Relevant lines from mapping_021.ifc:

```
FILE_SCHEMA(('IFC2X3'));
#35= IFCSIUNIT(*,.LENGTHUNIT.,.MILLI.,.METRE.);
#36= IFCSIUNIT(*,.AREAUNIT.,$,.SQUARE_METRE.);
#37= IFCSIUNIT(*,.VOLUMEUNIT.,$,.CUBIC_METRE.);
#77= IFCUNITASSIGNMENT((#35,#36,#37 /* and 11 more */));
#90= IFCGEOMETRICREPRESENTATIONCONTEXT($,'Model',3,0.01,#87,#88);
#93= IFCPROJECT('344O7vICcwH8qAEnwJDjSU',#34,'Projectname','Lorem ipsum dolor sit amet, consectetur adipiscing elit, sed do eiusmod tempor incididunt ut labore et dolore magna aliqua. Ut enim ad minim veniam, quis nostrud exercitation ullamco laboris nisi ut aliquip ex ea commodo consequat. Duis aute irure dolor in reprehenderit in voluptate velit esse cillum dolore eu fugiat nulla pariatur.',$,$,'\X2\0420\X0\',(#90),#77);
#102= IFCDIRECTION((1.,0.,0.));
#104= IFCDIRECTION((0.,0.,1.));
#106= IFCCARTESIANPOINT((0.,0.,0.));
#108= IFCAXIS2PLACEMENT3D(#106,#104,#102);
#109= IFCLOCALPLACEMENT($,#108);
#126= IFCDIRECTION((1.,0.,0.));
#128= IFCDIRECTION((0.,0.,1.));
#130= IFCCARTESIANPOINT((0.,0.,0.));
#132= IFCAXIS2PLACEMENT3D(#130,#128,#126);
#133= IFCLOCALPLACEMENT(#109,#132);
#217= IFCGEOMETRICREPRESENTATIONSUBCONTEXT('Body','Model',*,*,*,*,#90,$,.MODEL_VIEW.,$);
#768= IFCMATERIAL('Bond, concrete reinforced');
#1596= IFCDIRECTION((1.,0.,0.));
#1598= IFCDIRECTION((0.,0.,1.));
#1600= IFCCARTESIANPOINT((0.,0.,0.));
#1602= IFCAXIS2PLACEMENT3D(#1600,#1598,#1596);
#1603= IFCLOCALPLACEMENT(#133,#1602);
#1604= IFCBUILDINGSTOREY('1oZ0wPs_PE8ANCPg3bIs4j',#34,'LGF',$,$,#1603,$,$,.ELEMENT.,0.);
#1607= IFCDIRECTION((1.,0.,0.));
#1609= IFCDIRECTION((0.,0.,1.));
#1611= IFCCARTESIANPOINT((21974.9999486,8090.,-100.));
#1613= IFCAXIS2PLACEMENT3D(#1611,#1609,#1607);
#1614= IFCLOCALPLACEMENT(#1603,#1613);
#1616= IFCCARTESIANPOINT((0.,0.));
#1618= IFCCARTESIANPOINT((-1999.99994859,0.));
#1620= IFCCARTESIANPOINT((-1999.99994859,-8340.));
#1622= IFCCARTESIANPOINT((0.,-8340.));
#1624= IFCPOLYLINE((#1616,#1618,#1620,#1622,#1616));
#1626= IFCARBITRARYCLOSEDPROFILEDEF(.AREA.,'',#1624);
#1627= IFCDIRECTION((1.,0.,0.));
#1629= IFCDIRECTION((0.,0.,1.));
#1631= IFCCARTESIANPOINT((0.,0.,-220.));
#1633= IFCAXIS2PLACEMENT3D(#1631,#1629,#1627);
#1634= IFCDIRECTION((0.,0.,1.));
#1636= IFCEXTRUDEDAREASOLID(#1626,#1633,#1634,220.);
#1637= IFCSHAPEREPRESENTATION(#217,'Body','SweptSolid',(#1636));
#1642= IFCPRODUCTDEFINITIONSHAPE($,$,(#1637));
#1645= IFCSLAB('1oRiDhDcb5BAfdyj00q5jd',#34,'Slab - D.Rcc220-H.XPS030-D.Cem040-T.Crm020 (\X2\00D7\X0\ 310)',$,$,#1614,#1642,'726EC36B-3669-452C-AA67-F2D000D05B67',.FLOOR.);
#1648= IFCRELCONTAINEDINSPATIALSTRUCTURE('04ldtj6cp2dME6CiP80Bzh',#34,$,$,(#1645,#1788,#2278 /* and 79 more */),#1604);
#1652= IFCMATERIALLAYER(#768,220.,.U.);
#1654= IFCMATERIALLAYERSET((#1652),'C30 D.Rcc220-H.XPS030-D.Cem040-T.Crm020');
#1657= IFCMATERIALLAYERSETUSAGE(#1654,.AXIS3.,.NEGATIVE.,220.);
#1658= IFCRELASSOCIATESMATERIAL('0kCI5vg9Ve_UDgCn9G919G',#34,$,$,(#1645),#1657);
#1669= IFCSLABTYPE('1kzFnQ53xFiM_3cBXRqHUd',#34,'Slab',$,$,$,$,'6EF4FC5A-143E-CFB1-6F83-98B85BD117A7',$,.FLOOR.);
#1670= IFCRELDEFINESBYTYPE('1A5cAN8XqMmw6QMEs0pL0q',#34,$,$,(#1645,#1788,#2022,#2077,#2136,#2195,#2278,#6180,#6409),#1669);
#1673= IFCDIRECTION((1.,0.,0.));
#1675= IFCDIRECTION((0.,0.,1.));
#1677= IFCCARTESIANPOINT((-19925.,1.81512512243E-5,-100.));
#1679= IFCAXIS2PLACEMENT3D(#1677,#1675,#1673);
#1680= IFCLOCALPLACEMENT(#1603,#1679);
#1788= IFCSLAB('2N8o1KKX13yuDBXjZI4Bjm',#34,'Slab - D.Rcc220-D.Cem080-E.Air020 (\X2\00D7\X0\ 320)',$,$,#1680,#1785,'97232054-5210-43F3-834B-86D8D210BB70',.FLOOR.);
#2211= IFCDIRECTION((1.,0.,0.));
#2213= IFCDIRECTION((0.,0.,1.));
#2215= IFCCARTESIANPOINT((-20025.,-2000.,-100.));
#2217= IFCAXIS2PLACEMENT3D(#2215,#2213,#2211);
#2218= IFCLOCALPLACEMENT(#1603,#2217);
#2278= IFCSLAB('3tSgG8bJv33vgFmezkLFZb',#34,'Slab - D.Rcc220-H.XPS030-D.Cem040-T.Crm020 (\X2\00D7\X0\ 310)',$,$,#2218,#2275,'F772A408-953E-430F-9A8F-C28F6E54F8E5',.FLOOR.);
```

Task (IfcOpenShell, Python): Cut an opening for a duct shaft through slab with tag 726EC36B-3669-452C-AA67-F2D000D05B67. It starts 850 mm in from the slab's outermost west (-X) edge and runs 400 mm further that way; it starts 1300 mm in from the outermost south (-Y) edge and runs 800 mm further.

```python
import numpy as np
import ifcopenshell
import ifcopenshell.api.feature
import ifcopenshell.api.geometry
import ifcopenshell.api.root
import ifcopenshell.geom
import ifcopenshell.util.placement
import ifcopenshell.util.representation
import ifcopenshell.util.shape
import ifcopenshell.util.unit

model = ifcopenshell.open("mapping_021.ifc")
unit_scale = ifcopenshell.util.unit.calculate_unit_scale(model)
settings = ifcopenshell.geom.settings()


def volume(element):
    """Net volume in cubic metres, openings subtracted."""
    shape = ifcopenshell.geom.create_shape(settings, element)
    return ifcopenshell.util.shape.get_volume(shape.geometry)


slab = model.by_id(1645)
before = volume(slab)

# Extent in the slab's own axes, in metres. The edges named are its -X and -Y sides.
slab_shape = ifcopenshell.geom.create_shape(settings, slab)
vertices = ifcopenshell.util.shape.get_vertices(slab_shape.geometry)
x_min, y_min, bottom = vertices.min(axis=0)
top = vertices[:, 2].max()

opening = ifcopenshell.api.root.create_entity(model, ifc_class="IfcOpeningElement", name="Duct shaft opening")
context = ifcopenshell.util.representation.get_context(model, "Model", "Body", "MODEL_VIEW")
width, depth = 0.4, 0.8
outline = [(0.0, 0.0), (width, 0.0), (width, depth), (0.0, depth), (0.0, 0.0)]
# Overshoot both faces by 50 mm so the cut is clean.
shape = ifcopenshell.api.geometry.add_slab_representation(
    model, context=context, depth=top - bottom + 0.1, polyline=outline
)
ifcopenshell.api.geometry.assign_representation(model, product=opening, representation=shape)

matrix = ifcopenshell.util.placement.get_local_placement(slab.ObjectPlacement)
matrix[:, 3] = matrix @ np.append(np.array([x_min + 0.85, y_min + 1.3, bottom - 0.05]) / unit_scale, 1.0)
ifcopenshell.api.geometry.edit_object_placement(model, product=opening, matrix=matrix, is_si=False)
ifcopenshell.api.feature.add_feature(model, feature=opening, element=slab)

after = volume(slab)

print(f"slab volume {before:.3f} -> {after:.3f} m3")

model.write("mapping_021_v2.ifc")
```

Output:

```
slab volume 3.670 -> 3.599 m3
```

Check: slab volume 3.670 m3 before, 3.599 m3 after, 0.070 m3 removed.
